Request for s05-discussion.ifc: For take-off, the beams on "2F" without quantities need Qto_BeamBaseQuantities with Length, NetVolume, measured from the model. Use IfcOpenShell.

First a look at what the model holds.

```python
import ifcopenshell
import ifcopenshell.util.element
import ifcopenshell.util.unit

model = ifcopenshell.open("s05-discussion.ifc")
print(model.schema)
for unit_type in ("LENGTHUNIT", "AREAUNIT", "VOLUMEUNIT"):
    print(unit_type, ifcopenshell.util.unit.calculate_unit_scale(model, unit_type))
storey = next(s for s in model.by_type("IfcBuildingStorey") if s.Name == "2F")
beams = [e for e in ifcopenshell.util.element.get_decomposition(storey) if e.is_a("IfcBeam")]
for e in sorted(beams, key=lambda e: e.id()):
    print(e.id(), e.is_a(), e.Name, list(ifcopenshell.util.element.get_psets(e, qtos_only=True)), sep=" | ")
```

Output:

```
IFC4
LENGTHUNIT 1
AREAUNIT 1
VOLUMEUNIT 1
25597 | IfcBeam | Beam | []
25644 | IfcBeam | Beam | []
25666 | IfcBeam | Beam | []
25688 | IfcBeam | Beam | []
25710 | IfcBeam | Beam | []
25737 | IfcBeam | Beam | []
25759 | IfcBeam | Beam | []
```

```python
import ifcopenshell
import ifcopenshell.api.pset
import ifcopenshell.geom
import ifcopenshell.util.element
import ifcopenshell.util.shape
import ifcopenshell.util.unit

model = ifcopenshell.open("s05-discussion.ifc")
unit_scale = ifcopenshell.util.unit.calculate_unit_scale(model)
volume_scale = ifcopenshell.util.unit.calculate_unit_scale(model, "VOLUMEUNIT")
settings = ifcopenshell.geom.settings()

storey = next(s for s in model.by_type("IfcBuildingStorey") if s.Name == "2F")
beams = [e for e in ifcopenshell.util.element.get_decomposition(storey) if e.is_a("IfcBeam")]

for e in sorted(beams, key=lambda e: e.id()):
    if ifcopenshell.util.element.get_psets(e, qtos_only=True, should_inherit=False):
        continue
    # Geometry comes back in metres, in the element's own axes.
    shape = ifcopenshell.geom.create_shape(settings, e)
    values = {
        "Length": ifcopenshell.util.shape.get_max_xyz(shape.geometry) / unit_scale,
        "NetVolume": ifcopenshell.util.shape.get_volume(shape.geometry) / volume_scale,
    }
    qto = ifcopenshell.api.pset.add_qto(model, product=e, name="Qto_BeamBaseQuantities")
    ifcopenshell.api.pset.edit_qto(model, qto=qto, properties=values)
    print(e.id(), {k: round(v, 3) for k, v in values.items()})

model.write("s05-discussion_edited.ifc")
```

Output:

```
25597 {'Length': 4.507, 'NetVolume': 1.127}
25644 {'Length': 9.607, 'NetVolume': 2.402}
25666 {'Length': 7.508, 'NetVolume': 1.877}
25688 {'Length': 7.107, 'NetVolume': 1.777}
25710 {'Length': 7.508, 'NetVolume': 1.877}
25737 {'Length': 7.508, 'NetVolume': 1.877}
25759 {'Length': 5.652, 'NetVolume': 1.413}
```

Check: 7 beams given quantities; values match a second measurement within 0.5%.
